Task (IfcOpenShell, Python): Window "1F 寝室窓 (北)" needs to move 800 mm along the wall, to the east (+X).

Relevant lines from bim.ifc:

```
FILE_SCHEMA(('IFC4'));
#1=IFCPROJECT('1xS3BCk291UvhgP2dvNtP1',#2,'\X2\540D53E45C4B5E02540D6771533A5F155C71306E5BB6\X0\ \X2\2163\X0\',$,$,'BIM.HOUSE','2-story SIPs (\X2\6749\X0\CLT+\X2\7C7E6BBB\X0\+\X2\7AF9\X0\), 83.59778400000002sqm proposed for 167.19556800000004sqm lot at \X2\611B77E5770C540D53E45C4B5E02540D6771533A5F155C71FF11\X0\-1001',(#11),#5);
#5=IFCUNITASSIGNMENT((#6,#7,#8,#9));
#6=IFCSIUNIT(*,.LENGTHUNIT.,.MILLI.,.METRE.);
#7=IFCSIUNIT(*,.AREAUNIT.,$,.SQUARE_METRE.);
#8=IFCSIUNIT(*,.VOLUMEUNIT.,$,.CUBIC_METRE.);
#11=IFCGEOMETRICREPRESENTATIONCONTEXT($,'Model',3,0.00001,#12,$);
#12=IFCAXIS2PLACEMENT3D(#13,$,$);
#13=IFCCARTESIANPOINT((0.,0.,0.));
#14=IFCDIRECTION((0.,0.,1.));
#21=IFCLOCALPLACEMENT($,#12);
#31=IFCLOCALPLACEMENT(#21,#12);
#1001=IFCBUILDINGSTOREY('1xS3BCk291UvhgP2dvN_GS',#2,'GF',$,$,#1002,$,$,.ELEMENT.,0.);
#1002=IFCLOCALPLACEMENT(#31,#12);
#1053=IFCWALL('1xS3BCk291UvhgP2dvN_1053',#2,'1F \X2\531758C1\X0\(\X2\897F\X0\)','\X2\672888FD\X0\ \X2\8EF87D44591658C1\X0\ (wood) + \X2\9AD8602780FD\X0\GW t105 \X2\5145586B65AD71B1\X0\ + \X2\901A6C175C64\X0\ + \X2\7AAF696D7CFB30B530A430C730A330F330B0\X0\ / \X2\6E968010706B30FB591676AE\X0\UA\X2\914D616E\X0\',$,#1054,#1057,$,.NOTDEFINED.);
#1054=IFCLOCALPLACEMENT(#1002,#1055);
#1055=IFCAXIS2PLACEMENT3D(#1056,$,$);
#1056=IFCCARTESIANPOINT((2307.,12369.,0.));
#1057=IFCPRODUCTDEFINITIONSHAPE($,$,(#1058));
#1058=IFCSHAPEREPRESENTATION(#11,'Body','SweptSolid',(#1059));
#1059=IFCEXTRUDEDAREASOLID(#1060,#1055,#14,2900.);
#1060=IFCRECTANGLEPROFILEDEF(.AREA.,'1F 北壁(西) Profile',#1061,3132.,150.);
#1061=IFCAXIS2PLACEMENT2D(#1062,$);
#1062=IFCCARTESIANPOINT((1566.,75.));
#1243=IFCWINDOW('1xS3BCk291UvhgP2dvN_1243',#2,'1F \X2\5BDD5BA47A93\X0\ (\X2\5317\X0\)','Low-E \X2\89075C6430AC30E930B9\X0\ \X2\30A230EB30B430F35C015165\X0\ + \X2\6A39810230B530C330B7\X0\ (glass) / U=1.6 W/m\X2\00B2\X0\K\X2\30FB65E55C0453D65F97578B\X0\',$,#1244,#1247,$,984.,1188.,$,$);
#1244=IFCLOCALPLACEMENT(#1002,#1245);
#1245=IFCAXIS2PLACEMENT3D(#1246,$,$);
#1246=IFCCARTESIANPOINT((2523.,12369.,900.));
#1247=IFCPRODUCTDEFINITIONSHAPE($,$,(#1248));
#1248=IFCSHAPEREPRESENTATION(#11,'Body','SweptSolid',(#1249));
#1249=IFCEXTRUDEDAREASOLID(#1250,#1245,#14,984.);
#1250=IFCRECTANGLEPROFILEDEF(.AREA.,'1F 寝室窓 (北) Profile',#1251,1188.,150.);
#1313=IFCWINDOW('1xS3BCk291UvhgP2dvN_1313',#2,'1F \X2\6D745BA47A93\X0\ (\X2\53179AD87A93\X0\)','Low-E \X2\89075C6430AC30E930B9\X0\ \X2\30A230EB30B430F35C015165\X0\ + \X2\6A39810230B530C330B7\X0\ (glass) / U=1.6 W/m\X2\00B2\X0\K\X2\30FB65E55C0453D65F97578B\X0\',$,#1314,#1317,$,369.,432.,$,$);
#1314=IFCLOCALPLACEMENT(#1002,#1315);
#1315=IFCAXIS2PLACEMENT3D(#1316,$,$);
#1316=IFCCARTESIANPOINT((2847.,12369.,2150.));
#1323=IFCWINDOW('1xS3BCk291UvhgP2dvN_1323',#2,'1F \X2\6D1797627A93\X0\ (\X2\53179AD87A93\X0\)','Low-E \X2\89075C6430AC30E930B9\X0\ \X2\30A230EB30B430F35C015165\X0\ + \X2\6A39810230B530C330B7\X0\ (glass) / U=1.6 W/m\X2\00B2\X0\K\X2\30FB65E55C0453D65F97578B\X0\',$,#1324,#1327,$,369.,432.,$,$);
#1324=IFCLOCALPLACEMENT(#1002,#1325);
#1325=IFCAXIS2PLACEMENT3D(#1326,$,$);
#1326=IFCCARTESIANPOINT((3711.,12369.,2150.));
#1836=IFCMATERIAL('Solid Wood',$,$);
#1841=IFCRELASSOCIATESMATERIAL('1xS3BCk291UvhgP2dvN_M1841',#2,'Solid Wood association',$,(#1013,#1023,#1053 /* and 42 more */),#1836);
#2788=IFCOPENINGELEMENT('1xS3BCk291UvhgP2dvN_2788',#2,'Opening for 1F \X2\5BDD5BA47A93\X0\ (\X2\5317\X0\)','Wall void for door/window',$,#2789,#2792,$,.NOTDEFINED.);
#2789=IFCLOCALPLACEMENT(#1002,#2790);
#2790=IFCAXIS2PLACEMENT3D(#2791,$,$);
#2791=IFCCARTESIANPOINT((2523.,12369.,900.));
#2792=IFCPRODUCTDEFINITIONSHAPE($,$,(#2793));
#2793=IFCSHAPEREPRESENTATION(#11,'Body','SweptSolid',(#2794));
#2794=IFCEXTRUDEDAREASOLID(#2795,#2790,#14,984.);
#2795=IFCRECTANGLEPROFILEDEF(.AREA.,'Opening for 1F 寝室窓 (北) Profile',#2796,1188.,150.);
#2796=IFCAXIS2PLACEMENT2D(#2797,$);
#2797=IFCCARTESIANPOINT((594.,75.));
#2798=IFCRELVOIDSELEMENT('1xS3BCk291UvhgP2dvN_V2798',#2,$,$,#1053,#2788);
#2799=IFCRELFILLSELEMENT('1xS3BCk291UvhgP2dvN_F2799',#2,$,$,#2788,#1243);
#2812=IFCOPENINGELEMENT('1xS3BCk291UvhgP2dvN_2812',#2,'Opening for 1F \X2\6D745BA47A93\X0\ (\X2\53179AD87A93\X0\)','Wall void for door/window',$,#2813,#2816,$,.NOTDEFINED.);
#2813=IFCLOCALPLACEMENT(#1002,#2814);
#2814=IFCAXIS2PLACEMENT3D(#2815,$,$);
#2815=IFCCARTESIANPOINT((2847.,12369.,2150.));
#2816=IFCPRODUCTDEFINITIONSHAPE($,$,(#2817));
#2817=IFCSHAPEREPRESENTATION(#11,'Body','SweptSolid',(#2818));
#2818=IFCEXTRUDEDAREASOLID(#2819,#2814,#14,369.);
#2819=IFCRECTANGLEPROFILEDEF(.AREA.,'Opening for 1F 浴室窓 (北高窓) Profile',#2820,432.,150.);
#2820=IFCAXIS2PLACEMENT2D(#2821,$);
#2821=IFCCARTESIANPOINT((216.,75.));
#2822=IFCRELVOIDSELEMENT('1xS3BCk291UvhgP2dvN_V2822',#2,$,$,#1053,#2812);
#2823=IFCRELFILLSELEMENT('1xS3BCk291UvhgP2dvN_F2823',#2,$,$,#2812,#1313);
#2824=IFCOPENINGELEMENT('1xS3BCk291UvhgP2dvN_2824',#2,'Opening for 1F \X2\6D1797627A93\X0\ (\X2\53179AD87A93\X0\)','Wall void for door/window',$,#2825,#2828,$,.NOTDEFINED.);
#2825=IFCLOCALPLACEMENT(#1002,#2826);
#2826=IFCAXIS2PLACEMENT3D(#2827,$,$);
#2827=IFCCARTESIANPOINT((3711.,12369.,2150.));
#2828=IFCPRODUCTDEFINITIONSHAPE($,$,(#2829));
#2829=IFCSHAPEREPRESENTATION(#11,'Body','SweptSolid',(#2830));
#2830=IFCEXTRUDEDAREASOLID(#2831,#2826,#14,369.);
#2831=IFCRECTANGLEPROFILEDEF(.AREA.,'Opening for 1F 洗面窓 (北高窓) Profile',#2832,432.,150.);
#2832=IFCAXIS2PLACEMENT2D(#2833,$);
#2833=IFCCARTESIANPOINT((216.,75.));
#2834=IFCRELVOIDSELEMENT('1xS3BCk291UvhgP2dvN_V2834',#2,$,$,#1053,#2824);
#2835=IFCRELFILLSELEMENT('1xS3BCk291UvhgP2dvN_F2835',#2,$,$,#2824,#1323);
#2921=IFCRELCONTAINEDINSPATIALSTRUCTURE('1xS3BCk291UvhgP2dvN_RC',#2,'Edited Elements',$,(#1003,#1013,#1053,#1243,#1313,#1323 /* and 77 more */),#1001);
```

```python
import ifcopenshell
import ifcopenshell.api.geometry
import ifcopenshell.util.placement

model = ifcopenshell.open("bim.ifc")

window = model.by_guid("1xS3BCk291UvhgP2dvN_1243")
opening = window.FillsVoids[0].RelatingOpeningElement
wall = opening.VoidsElements[0].RelatingBuildingElement

wall_matrix = ifcopenshell.util.placement.get_local_placement(wall.ObjectPlacement)
shift = wall_matrix[:3, 0] * 800.0
before = ifcopenshell.util.placement.get_local_placement(window.ObjectPlacement)[:3, 3].copy()

# The window is not placed relative to its opening, so move both.
for product in (opening, window):
    matrix = ifcopenshell.util.placement.get_local_placement(product.ObjectPlacement)
    matrix[:3, 3] += shift
    ifcopenshell.api.geometry.edit_object_placement(model, product=product, matrix=matrix, is_si=False)

after = ifcopenshell.util.placement.get_local_placement(window.ObjectPlacement)[:3, 3]
print("window moved by", (after - before).round(3) + 0.0)

model.write("bim_updated.ifc")
```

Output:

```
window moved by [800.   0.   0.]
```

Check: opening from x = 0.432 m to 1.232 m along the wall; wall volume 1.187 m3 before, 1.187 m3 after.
